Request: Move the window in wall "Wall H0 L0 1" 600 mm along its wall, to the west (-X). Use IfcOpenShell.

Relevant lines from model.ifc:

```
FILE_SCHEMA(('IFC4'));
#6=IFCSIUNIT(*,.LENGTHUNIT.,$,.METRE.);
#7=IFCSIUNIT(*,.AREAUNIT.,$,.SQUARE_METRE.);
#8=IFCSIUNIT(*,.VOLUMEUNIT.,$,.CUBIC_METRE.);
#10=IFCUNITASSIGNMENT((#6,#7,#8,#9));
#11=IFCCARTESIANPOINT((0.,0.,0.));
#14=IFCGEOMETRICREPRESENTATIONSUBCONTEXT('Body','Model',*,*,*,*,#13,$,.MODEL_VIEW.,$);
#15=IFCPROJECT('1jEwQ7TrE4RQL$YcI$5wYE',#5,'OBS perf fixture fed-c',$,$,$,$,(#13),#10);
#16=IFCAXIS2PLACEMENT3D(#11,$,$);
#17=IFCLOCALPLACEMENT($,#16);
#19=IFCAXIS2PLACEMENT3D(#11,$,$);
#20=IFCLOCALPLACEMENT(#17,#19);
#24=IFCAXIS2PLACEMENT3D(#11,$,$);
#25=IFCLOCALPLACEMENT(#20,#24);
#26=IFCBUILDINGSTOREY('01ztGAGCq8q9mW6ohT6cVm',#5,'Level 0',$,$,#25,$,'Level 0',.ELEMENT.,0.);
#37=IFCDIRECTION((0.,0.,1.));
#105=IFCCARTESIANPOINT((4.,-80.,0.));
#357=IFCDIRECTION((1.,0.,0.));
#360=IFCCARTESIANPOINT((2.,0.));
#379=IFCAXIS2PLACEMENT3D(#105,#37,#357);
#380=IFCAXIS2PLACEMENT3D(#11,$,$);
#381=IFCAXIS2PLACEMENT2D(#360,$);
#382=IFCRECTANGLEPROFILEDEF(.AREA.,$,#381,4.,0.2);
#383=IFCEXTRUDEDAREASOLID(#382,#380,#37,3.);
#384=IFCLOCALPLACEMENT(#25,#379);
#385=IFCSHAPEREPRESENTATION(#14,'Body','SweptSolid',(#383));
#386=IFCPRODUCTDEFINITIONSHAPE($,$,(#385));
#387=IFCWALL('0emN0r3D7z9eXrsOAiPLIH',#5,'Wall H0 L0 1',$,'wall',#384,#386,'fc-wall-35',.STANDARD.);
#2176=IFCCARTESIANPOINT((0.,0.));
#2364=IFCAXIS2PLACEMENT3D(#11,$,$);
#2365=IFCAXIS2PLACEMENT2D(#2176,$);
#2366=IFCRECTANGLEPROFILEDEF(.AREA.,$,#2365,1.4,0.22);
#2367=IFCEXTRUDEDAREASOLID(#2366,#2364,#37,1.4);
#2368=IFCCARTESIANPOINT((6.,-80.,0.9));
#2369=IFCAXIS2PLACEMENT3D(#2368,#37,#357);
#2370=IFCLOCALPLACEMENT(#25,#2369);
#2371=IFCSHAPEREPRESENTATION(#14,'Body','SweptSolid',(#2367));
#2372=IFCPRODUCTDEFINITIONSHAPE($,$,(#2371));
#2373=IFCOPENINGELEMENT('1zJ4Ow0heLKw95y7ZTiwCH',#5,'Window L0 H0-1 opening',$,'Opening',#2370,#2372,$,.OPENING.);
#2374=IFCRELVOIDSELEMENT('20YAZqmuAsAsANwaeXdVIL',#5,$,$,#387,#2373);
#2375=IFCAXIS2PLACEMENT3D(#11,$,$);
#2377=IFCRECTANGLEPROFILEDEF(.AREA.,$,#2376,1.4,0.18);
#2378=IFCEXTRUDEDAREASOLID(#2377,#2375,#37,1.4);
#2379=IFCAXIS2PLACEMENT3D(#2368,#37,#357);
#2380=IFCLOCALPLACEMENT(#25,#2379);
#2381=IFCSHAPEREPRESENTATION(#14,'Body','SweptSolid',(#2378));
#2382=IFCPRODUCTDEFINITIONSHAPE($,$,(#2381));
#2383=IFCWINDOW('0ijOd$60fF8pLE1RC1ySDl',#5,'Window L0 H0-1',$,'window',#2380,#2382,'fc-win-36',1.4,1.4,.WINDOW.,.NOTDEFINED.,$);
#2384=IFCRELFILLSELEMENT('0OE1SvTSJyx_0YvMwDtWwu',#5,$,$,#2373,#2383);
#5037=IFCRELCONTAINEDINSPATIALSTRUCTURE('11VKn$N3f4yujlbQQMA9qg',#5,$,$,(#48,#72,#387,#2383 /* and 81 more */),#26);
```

```python
import ifcopenshell
import ifcopenshell.api.geometry
import ifcopenshell.util.placement

model = ifcopenshell.open("model.ifc")

window = model.by_guid("0ijOd$60fF8pLE1RC1ySDl")
opening = window.FillsVoids[0].RelatingOpeningElement
wall = opening.VoidsElements[0].RelatingBuildingElement

wall_matrix = ifcopenshell.util.placement.get_local_placement(wall.ObjectPlacement)
shift = wall_matrix[:3, 0] * -0.6
before = ifcopenshell.util.placement.get_local_placement(window.ObjectPlacement)[:3, 3].copy()

# The window is not placed relative to its opening, so move both.
for product in (opening, window):
    matrix = ifcopenshell.util.placement.get_local_placement(product.ObjectPlacement)
    matrix[:3, 3] += shift
    ifcopenshell.api.geometry.edit_object_placement(model, product=product, matrix=matrix, is_si=False)

after = ifcopenshell.util.placement.get_local_placement(window.ObjectPlacement)[:3, 3]
print("window moved by", (after - before).round(3) + 0.0)

model.write("model-out.ifc")
```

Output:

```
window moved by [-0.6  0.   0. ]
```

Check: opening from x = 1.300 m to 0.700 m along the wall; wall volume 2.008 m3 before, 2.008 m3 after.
